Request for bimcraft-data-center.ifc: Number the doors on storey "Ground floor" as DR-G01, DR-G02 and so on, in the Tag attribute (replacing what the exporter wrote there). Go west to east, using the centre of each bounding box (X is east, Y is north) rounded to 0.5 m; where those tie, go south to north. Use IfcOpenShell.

First a look at what the model holds.

```python
import ifcopenshell
import ifcopenshell.util.element
import ifcopenshell.util.placement

model = ifcopenshell.open("bimcraft-data-center.ifc")
print(model.schema)
storey = next(s for s in model.by_type("IfcBuildingStorey") if s.Name == "Ground floor")
doors = [e for e in ifcopenshell.util.element.get_decomposition(storey) if e.is_a("IfcDoor")]
for e in sorted(doors, key=lambda e: e.id()):
    origin = ifcopenshell.util.placement.get_local_placement(e.ObjectPlacement)[:3, 3]
    print(e.id(), e.Tag, e.Name, origin.round(2) + 0.0, sep=" | ")
```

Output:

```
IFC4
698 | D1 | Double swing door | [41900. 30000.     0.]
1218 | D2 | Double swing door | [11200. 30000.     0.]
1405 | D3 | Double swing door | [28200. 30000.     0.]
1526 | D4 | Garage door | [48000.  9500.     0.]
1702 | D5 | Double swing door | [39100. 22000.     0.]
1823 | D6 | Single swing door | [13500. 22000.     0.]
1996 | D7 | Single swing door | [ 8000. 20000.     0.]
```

```python
import ifcopenshell
import ifcopenshell.geom
import ifcopenshell.util.element
import ifcopenshell.util.shape

model = ifcopenshell.open("bimcraft-data-center.ifc")
settings = ifcopenshell.geom.settings()
settings.set("use-world-coords", True)


def centre(element):
    shape = ifcopenshell.geom.create_shape(settings, element)
    return ifcopenshell.util.shape.get_bbox_centroid(shape.geometry)


storey = next(s for s in model.by_type("IfcBuildingStorey") if s.Name == "Ground floor")
doors = [e for e in ifcopenshell.util.element.get_decomposition(storey) if e.is_a("IfcDoor")]

# Insertion points can sit at a corner or the storey origin, so sort by the geometry (in metres).
centres = {e: centre(e) for e in doors}
doors.sort(key=lambda e: (round(centres[e][0] / 0.5), centres[e][1]))

for i, e in enumerate(doors, start=1):
    number = f"DR-G{i:02d}"
    e.Tag = number
    print(e.id(), number)

model.write("bimcraft-data-center_v2.ifc")
```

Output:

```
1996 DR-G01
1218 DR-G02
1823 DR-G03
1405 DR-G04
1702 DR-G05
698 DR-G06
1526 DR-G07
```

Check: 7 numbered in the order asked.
